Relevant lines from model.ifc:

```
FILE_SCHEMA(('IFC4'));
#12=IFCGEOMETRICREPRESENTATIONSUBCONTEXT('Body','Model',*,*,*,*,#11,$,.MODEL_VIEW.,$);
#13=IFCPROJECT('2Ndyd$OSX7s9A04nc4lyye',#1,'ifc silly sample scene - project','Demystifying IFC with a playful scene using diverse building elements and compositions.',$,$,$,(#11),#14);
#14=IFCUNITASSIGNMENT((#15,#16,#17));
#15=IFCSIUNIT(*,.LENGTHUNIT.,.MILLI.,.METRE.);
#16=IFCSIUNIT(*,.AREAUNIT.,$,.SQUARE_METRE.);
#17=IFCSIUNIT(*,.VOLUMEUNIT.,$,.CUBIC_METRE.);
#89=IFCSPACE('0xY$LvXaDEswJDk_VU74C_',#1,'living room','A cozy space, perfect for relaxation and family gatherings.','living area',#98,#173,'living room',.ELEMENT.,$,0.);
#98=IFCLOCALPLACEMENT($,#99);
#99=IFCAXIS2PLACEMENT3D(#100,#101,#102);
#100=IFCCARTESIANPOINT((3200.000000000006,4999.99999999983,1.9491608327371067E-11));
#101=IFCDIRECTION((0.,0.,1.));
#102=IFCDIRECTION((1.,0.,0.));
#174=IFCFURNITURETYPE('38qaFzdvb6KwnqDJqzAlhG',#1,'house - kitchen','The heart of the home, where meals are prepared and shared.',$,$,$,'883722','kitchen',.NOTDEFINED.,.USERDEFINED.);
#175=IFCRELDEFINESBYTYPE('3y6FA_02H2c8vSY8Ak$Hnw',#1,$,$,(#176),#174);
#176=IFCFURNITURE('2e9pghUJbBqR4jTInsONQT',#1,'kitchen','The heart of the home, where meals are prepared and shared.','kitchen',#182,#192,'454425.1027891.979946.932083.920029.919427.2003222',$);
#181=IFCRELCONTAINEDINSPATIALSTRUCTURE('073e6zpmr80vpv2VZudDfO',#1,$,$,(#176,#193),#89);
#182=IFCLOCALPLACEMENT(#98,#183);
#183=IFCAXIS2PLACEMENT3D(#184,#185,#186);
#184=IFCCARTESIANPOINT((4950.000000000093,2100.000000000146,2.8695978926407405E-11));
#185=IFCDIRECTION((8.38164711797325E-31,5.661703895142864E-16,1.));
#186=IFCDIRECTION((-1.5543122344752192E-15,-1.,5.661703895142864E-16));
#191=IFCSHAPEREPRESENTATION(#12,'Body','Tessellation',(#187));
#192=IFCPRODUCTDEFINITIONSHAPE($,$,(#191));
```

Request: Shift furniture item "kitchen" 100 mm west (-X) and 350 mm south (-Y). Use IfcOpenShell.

```python
import ifcopenshell
import ifcopenshell.api.geometry
import ifcopenshell.util.placement

model = ifcopenshell.open("model.ifc")

item = model.by_guid("2e9pghUJbBqR4jTInsONQT")
matrix = ifcopenshell.util.placement.get_local_placement(item.ObjectPlacement)
matrix[0, 3] -= 100.0
matrix[1, 3] -= 350.0
ifcopenshell.api.geometry.edit_object_placement(model, product=item, matrix=matrix, is_si=False)

print(ifcopenshell.util.placement.get_local_placement(item.ObjectPlacement).round(3) + 0.0)

model.write("model_updated.ifc")
```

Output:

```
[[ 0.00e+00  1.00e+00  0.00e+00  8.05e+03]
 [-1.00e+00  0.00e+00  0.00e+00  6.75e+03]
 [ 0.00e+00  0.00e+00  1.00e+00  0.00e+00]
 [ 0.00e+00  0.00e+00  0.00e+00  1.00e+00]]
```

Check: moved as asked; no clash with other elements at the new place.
